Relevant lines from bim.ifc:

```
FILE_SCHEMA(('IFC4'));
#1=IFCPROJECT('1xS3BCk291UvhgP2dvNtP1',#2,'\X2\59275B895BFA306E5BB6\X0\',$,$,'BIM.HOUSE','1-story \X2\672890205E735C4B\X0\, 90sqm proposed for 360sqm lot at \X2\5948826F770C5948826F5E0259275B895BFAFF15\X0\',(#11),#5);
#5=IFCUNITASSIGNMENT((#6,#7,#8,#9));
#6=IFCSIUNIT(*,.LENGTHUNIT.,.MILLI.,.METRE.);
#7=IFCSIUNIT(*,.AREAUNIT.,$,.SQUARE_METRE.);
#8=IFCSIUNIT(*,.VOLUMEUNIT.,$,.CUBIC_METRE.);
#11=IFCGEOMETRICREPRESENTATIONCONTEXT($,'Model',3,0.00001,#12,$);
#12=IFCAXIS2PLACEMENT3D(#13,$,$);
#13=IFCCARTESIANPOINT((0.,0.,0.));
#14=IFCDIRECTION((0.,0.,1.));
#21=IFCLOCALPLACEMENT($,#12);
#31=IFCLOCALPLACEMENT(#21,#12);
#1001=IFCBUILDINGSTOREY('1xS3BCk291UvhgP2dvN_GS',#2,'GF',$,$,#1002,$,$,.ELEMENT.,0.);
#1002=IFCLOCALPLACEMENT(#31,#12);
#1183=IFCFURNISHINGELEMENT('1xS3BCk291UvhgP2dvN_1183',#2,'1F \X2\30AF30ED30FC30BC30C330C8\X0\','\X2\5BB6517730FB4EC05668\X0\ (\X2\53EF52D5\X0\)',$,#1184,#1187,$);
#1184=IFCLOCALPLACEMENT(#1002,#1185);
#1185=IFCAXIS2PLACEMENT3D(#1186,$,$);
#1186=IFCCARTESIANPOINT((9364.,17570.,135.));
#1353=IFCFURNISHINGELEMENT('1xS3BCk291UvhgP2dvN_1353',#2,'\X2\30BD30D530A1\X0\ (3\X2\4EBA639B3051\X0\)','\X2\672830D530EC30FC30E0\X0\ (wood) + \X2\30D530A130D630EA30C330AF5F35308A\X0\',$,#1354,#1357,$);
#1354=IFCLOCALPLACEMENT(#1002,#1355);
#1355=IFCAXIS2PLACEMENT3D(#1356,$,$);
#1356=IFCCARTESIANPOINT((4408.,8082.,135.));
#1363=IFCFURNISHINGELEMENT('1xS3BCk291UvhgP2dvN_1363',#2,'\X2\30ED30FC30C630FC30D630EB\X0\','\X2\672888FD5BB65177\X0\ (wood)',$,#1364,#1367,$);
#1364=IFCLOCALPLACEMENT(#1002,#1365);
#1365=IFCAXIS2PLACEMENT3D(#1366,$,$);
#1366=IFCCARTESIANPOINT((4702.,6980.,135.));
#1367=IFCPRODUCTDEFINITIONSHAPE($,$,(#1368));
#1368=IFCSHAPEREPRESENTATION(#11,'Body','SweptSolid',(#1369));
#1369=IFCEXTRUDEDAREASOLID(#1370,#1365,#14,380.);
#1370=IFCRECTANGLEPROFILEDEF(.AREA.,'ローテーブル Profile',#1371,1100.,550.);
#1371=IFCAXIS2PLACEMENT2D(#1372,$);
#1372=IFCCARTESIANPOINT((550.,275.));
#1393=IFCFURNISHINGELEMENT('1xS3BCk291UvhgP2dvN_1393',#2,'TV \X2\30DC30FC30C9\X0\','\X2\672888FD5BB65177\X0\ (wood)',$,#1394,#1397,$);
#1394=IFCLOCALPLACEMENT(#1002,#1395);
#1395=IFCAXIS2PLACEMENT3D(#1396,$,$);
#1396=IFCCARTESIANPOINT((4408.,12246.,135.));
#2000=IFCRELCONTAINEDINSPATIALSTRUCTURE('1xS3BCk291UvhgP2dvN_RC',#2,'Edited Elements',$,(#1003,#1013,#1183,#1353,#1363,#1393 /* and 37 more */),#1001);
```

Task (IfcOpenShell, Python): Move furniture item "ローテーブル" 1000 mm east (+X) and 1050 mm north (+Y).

```python
import ifcopenshell
import ifcopenshell.api.geometry
import ifcopenshell.util.placement

model = ifcopenshell.open("bim.ifc")

item = model.by_id(1363)
matrix = ifcopenshell.util.placement.get_local_placement(item.ObjectPlacement)
matrix[0, 3] += 1000.0
matrix[1, 3] += 1050.0
ifcopenshell.api.geometry.edit_object_placement(model, product=item, matrix=matrix, is_si=False)

print(ifcopenshell.util.placement.get_local_placement(item.ObjectPlacement).round(3) + 0.0)

model.write("bim_edited.ifc")
```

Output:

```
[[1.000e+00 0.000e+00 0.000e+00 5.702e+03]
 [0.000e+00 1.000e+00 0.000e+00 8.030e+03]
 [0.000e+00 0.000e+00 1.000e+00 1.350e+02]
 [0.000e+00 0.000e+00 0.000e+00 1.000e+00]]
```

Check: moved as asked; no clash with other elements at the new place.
